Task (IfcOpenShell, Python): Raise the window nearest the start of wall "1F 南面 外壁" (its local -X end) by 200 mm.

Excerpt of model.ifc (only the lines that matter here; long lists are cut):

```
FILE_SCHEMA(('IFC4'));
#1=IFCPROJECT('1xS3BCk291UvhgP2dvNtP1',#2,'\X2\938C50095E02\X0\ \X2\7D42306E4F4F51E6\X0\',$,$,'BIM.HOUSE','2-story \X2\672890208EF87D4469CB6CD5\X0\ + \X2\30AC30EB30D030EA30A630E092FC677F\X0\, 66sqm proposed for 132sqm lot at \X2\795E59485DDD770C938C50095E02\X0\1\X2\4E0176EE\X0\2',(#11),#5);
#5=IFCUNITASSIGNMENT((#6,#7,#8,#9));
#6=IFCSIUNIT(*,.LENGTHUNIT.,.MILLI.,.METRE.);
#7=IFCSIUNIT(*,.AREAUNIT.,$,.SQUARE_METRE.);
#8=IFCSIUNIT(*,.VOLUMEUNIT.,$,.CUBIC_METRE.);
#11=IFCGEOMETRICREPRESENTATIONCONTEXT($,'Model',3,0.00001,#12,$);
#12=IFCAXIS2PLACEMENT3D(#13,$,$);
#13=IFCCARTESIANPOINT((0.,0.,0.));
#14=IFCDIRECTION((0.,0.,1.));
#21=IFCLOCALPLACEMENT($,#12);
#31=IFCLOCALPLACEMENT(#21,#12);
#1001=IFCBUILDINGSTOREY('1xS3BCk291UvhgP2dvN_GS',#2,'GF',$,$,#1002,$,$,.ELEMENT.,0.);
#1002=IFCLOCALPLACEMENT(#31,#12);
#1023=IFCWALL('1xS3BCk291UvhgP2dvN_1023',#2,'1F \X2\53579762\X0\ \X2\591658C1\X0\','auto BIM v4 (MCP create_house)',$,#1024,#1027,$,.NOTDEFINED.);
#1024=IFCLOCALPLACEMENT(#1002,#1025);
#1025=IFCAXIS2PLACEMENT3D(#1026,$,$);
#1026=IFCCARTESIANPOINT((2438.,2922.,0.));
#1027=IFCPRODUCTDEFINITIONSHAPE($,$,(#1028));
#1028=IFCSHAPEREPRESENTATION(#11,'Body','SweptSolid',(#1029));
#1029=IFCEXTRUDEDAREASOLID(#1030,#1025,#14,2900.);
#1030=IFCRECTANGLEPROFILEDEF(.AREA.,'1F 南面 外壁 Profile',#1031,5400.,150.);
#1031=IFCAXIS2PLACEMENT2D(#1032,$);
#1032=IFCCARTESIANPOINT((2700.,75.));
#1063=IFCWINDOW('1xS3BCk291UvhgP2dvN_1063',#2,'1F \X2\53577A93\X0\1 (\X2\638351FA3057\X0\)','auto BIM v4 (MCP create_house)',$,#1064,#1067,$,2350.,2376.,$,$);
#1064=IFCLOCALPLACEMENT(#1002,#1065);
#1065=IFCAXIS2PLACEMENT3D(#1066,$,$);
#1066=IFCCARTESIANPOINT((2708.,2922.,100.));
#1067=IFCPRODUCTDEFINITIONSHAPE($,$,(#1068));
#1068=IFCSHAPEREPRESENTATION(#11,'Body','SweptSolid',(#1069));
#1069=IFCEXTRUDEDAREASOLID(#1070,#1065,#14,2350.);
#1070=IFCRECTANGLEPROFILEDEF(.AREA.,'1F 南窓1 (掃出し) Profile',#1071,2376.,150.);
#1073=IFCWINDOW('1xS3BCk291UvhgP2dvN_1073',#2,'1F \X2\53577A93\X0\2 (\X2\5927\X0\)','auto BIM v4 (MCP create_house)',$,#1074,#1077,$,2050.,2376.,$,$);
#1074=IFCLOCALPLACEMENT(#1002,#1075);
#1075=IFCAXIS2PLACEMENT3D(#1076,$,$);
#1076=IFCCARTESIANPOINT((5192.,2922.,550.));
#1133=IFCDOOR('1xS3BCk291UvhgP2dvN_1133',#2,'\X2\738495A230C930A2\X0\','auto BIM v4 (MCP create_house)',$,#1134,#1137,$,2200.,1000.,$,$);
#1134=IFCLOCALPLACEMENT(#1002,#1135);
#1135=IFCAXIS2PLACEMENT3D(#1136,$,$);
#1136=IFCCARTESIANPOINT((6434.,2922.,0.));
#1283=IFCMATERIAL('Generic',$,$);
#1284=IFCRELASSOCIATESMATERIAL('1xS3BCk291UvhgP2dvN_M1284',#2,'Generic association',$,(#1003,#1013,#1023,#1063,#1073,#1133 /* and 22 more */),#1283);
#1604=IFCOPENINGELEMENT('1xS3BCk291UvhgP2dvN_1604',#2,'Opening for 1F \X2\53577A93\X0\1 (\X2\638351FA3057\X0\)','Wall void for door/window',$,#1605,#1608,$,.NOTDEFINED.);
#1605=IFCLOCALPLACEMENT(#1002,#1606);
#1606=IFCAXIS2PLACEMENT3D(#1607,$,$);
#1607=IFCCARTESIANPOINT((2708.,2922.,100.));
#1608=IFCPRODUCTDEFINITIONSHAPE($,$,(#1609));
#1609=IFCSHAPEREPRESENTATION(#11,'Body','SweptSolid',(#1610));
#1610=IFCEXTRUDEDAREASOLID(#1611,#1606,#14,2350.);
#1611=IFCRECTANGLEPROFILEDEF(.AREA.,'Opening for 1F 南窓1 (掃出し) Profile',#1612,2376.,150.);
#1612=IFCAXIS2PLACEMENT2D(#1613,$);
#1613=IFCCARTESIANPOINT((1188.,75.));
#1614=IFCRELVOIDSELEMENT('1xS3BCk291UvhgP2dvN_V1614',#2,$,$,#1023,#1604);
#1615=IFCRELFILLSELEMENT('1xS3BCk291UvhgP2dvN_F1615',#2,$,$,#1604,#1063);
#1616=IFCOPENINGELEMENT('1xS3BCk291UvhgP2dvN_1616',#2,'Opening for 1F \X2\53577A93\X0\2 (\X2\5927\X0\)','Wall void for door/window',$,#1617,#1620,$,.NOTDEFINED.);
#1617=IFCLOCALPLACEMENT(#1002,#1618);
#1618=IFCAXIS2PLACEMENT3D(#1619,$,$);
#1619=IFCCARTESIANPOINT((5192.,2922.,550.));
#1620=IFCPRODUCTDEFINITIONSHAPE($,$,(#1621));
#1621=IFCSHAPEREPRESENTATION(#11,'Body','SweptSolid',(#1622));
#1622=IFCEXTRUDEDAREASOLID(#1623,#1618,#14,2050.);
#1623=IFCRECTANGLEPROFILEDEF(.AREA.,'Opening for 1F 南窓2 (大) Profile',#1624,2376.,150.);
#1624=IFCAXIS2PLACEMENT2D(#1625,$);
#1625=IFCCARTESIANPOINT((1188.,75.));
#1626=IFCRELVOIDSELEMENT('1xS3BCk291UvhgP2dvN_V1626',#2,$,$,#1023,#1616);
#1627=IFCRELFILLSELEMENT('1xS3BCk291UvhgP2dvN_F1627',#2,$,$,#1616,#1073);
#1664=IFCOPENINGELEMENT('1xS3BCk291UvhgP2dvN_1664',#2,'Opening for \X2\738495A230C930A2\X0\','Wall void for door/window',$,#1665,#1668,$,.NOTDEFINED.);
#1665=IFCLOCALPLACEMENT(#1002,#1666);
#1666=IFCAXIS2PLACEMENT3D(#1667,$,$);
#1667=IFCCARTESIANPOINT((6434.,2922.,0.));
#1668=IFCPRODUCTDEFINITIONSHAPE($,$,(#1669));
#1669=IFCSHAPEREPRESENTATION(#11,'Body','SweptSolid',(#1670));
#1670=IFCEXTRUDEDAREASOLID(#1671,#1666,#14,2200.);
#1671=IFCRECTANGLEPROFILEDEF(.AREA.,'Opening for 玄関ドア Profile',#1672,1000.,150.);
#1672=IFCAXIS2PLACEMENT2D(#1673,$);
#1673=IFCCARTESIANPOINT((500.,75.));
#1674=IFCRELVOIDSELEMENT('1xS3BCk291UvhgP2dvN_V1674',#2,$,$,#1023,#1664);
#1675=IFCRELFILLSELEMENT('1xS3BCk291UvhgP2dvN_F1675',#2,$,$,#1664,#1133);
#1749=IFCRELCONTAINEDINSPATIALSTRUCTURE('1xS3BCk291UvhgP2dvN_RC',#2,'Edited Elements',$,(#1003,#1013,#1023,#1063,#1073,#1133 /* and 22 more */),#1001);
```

```python
import numpy as np
import ifcopenshell
import ifcopenshell.api.geometry
import ifcopenshell.util.placement
import ifcopenshell.util.unit

model = ifcopenshell.open("model.ifc")
unit_scale = ifcopenshell.util.unit.calculate_unit_scale(model)

window = model.by_guid("1xS3BCk291UvhgP2dvN_1063")
opening = window.FillsVoids[0].RelatingOpeningElement
dz = 0.2 / unit_scale

shift = np.array([0.0, 0.0, dz])
# The window is not placed relative to its opening, so move both.
for product in (opening, window):
    matrix = ifcopenshell.util.placement.get_local_placement(product.ObjectPlacement)
    matrix[:3, 3] += shift
    ifcopenshell.api.geometry.edit_object_placement(model, product=product, matrix=matrix, is_si=False)

print(f"moved by {dz * unit_scale:+.3f} m")

model.write("model_rev.ifc")
```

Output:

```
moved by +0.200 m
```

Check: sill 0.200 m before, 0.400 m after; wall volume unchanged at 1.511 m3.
